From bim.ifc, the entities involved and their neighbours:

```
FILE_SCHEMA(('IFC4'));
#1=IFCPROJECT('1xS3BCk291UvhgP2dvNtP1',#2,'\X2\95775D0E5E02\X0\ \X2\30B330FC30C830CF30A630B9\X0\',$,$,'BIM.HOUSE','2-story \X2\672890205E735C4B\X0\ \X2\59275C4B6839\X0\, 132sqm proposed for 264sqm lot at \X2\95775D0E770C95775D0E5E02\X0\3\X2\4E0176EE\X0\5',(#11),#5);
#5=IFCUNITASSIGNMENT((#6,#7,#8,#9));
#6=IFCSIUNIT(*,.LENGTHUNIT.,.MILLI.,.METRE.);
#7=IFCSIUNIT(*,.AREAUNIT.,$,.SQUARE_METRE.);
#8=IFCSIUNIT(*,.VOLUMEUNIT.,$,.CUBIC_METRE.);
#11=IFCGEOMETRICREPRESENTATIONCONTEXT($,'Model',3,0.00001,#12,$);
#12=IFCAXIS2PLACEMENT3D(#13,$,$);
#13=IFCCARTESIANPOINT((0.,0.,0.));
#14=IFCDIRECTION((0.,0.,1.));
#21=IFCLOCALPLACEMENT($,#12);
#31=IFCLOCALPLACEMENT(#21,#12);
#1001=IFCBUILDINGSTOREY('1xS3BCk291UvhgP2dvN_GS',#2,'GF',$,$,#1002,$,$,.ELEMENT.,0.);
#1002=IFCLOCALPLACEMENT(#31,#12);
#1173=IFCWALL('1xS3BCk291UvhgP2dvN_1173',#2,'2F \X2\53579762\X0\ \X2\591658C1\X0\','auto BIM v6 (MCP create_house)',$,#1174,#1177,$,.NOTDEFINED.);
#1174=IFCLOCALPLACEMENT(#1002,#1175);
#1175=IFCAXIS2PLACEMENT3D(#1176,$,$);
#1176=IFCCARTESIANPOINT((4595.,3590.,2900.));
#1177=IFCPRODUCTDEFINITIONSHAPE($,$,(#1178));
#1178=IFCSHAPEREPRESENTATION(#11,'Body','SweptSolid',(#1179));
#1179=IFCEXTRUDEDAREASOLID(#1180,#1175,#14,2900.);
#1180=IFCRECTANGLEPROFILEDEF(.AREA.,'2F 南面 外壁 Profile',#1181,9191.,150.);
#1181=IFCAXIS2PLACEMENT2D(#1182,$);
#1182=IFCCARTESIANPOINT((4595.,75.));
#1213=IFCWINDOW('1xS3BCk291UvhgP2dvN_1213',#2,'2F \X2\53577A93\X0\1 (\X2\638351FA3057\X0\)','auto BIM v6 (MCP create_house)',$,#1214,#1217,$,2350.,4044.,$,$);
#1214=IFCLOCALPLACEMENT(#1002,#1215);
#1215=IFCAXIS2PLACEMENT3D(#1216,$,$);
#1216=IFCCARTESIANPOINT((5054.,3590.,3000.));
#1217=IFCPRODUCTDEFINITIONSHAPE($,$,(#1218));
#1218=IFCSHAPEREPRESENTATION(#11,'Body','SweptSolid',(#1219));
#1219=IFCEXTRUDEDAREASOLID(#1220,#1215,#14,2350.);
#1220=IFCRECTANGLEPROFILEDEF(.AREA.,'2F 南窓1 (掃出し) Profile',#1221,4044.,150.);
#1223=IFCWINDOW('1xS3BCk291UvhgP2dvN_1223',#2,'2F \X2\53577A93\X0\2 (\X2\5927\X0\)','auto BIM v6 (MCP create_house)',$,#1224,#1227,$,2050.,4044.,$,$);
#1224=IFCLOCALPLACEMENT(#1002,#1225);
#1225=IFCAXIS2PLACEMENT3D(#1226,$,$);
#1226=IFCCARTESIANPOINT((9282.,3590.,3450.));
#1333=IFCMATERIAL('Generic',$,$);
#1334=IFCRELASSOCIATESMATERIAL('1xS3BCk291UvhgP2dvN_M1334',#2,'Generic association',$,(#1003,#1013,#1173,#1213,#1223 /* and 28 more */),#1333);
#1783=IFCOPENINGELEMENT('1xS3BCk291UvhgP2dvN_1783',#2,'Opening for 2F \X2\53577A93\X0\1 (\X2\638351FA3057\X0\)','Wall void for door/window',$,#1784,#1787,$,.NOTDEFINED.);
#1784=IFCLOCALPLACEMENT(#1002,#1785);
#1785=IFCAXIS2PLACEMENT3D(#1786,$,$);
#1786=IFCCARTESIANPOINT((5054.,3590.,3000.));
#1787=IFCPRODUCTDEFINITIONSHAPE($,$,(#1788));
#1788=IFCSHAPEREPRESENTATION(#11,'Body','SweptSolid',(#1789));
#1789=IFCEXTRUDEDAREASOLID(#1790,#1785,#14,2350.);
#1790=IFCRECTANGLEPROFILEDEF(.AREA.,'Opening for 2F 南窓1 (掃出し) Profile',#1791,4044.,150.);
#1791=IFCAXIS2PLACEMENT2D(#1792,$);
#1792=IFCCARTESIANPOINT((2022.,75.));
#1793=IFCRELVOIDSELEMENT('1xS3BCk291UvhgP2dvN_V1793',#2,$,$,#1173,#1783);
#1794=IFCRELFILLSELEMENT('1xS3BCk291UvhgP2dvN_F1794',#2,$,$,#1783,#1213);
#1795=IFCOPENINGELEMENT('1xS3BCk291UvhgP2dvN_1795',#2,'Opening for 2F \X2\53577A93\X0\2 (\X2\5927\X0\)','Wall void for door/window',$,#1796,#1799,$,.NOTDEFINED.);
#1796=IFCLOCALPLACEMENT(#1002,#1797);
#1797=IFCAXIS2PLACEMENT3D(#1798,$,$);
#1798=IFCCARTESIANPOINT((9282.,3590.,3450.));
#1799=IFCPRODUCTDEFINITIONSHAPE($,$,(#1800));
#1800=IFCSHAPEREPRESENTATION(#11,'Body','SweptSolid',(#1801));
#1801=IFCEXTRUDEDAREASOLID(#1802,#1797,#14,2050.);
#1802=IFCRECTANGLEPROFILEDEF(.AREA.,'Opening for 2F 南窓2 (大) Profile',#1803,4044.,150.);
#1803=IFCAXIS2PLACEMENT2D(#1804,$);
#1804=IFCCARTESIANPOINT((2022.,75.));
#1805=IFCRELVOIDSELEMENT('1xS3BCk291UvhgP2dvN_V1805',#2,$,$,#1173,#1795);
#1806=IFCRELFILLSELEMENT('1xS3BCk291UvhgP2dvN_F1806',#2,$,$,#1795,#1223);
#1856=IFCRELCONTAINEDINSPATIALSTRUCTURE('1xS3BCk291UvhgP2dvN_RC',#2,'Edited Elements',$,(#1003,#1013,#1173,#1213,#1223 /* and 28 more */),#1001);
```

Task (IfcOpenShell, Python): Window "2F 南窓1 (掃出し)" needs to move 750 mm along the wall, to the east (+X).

```python
import ifcopenshell
import ifcopenshell.api.geometry
import ifcopenshell.util.placement

model = ifcopenshell.open("bim.ifc")

window = model.by_guid("1xS3BCk291UvhgP2dvN_1213")
opening = window.FillsVoids[0].RelatingOpeningElement
wall = opening.VoidsElements[0].RelatingBuildingElement

wall_matrix = ifcopenshell.util.placement.get_local_placement(wall.ObjectPlacement)
shift = wall_matrix[:3, 0] * 750.0
before = ifcopenshell.util.placement.get_local_placement(window.ObjectPlacement)[:3, 3].copy()

# The window is not placed relative to its opening, so move both.
for product in (opening, window):
    matrix = ifcopenshell.util.placement.get_local_placement(product.ObjectPlacement)
    matrix[:3, 3] += shift
    ifcopenshell.api.geometry.edit_object_placement(model, product=product, matrix=matrix, is_si=False)

after = ifcopenshell.util.placement.get_local_placement(window.ObjectPlacement)[:3, 3]
print("window moved by", (after - before).round(3) + 0.0)

model.write("bim_updated.ifc")
```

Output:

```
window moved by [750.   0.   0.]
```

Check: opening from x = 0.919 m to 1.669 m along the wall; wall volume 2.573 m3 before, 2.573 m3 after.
